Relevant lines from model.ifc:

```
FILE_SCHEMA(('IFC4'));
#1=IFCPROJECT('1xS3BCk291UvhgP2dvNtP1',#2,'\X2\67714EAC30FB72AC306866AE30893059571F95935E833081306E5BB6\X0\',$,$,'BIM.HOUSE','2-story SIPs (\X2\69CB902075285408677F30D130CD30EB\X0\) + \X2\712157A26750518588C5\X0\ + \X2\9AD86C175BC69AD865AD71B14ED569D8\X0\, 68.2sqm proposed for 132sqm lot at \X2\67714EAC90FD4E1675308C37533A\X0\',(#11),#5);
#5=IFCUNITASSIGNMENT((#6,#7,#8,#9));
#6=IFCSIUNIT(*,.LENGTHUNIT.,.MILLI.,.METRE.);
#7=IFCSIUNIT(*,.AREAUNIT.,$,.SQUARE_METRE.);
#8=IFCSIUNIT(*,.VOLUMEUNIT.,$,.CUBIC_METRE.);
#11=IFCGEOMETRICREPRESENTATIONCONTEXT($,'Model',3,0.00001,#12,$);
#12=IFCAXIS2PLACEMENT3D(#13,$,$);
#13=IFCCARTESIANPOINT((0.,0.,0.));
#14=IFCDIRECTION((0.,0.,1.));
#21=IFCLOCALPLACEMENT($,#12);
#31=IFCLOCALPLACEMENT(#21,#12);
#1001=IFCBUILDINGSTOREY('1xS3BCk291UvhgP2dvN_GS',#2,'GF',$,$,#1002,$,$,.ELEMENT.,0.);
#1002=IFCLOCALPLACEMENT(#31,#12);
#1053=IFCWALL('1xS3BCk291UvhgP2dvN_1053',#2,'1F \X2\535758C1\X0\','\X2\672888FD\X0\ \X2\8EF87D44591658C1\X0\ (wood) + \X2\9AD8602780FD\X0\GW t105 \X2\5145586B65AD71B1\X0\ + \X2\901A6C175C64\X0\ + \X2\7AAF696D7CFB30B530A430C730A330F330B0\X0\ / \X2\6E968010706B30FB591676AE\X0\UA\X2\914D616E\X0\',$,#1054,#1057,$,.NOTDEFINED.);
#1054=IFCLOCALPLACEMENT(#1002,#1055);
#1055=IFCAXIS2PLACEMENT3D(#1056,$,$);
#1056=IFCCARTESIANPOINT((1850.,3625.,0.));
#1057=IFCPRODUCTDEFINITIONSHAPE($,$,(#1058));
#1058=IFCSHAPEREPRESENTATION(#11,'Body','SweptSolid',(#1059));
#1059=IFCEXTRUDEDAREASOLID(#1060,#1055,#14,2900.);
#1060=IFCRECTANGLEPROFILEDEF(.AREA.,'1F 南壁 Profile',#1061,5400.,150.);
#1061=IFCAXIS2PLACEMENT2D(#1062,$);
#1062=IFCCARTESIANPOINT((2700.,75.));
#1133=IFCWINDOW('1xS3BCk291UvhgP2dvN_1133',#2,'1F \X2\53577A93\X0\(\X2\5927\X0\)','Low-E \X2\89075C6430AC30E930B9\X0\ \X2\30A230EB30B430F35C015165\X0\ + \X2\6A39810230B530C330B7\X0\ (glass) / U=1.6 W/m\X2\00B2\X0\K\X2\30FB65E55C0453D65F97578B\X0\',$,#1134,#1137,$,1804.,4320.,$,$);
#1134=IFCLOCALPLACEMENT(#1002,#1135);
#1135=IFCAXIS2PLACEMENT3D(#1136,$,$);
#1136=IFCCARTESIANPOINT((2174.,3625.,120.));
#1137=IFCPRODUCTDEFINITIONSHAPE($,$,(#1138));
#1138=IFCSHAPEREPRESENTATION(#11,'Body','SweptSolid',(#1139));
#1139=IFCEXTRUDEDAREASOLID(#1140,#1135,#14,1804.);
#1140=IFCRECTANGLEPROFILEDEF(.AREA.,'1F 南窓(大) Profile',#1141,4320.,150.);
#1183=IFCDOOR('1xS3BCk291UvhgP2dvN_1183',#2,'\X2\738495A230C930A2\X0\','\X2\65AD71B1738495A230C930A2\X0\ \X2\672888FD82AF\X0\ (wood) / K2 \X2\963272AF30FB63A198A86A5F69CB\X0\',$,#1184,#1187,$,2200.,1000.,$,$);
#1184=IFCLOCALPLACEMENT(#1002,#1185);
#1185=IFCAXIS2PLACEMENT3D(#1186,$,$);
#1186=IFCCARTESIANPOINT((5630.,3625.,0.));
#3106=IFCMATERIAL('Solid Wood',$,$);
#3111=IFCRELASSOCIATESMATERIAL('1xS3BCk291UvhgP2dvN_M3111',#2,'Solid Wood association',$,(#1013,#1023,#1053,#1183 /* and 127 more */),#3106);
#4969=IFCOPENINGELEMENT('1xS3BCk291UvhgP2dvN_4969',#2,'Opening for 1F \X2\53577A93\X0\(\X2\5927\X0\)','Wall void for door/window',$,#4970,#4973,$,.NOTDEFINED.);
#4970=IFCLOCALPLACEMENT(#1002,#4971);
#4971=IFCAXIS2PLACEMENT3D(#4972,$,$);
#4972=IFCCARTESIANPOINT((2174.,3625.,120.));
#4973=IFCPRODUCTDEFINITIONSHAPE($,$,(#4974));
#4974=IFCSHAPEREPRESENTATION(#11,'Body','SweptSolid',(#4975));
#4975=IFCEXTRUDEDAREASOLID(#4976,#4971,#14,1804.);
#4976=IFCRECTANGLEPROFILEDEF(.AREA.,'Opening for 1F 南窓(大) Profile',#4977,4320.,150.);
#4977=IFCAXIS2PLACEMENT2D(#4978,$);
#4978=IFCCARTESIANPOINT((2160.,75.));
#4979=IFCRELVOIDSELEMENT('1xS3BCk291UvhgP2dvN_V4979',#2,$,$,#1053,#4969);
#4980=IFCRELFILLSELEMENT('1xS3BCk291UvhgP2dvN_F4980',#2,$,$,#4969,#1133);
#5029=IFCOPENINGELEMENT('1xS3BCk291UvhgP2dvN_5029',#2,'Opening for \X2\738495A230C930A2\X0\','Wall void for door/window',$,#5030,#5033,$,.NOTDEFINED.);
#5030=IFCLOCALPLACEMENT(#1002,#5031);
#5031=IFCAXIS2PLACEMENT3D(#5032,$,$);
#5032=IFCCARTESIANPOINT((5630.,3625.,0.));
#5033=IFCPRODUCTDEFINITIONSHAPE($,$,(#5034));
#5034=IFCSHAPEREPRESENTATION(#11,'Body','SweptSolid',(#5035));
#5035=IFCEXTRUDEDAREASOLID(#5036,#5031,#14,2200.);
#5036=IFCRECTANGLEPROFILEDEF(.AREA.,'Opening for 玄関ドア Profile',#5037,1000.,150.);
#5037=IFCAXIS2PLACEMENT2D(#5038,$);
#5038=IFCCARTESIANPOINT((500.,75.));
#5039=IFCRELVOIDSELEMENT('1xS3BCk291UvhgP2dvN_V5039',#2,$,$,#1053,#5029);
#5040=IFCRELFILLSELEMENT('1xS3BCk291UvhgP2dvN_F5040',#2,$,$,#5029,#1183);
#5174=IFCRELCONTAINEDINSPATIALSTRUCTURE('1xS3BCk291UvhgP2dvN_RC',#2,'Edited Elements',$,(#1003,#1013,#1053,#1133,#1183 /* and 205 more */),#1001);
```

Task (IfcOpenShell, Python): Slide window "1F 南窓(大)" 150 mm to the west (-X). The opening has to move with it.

```python
import ifcopenshell
import ifcopenshell.api.geometry
import ifcopenshell.util.placement
import ifcopenshell.util.unit

model = ifcopenshell.open("model.ifc")
unit_scale = ifcopenshell.util.unit.calculate_unit_scale(model)

window = model.by_id(1133)
opening = window.FillsVoids[0].RelatingOpeningElement
wall = opening.VoidsElements[0].RelatingBuildingElement

wall_matrix = ifcopenshell.util.placement.get_local_placement(wall.ObjectPlacement)
shift = wall_matrix[:3, 0] * -0.15 / unit_scale
before = ifcopenshell.util.placement.get_local_placement(window.ObjectPlacement)[:3, 3].copy()

# The window is not placed relative to its opening, so move both.
for product in (opening, window):
    matrix = ifcopenshell.util.placement.get_local_placement(product.ObjectPlacement)
    matrix[:3, 3] += shift
    ifcopenshell.api.geometry.edit_object_placement(model, product=product, matrix=matrix, is_si=False)

after = ifcopenshell.util.placement.get_local_placement(window.ObjectPlacement)[:3, 3]
print("window moved by", (after - before).round(3) + 0.0)

model.write("model_rev.ifc")
```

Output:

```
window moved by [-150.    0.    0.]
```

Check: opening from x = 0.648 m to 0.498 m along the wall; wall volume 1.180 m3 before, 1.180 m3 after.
